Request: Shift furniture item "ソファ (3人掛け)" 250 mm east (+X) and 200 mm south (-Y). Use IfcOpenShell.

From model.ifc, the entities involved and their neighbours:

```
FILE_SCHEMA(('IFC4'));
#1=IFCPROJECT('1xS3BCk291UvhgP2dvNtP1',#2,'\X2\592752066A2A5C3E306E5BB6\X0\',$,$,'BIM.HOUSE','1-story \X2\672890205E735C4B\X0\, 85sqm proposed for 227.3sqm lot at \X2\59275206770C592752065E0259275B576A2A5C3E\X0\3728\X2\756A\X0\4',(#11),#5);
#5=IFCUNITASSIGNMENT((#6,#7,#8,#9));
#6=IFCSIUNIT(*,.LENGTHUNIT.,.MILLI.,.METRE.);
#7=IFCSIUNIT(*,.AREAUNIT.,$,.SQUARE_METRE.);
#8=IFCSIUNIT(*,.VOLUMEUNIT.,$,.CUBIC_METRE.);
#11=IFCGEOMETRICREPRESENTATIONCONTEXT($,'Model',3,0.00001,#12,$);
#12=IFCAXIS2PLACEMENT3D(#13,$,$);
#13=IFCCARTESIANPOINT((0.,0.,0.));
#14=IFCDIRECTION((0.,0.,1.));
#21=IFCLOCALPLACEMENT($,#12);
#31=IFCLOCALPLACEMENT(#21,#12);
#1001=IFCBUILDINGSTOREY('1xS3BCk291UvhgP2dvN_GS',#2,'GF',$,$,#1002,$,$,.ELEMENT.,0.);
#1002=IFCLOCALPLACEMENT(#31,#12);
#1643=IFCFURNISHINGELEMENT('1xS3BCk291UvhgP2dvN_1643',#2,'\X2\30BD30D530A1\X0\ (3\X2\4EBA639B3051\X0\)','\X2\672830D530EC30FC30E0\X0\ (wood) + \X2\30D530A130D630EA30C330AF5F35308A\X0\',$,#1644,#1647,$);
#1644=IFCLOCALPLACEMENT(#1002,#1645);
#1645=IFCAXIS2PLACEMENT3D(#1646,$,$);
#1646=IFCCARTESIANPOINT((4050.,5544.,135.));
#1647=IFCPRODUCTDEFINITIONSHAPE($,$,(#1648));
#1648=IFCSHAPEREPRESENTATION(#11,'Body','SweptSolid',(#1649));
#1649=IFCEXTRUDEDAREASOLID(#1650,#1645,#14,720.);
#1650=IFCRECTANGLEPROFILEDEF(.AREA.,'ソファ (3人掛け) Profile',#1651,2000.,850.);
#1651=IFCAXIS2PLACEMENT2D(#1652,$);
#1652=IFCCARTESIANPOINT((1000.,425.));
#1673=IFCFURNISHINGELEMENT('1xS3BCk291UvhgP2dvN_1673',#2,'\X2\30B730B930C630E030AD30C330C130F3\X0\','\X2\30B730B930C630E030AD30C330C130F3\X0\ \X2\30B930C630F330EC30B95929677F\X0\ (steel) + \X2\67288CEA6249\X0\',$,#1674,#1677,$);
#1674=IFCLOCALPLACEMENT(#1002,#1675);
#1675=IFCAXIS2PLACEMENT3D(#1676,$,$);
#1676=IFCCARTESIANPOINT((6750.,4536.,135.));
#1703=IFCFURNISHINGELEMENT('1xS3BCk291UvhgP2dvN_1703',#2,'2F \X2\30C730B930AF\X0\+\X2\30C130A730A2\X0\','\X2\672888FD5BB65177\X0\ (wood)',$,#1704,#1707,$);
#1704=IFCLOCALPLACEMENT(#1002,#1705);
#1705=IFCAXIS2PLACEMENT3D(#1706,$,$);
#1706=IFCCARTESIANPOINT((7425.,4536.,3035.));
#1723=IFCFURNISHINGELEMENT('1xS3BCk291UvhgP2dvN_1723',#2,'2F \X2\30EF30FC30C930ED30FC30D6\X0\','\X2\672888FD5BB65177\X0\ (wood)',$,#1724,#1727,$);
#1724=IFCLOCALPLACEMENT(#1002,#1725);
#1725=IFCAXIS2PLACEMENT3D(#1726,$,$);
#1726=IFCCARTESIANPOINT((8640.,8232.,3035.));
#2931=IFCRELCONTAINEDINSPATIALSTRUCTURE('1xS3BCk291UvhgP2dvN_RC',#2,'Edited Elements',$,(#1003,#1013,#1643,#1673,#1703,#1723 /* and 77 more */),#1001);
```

```python
import ifcopenshell
import ifcopenshell.api.geometry
import ifcopenshell.util.placement
import ifcopenshell.util.unit

model = ifcopenshell.open("model.ifc")
unit_scale = ifcopenshell.util.unit.calculate_unit_scale(model)

item = model.by_id(1643)
matrix = ifcopenshell.util.placement.get_local_placement(item.ObjectPlacement)
matrix[0, 3] += 0.25 / unit_scale
matrix[1, 3] -= 0.2 / unit_scale
ifcopenshell.api.geometry.edit_object_placement(model, product=item, matrix=matrix, is_si=False)

print(ifcopenshell.util.placement.get_local_placement(item.ObjectPlacement).round(3) + 0.0)

model.write("model_edited.ifc")
```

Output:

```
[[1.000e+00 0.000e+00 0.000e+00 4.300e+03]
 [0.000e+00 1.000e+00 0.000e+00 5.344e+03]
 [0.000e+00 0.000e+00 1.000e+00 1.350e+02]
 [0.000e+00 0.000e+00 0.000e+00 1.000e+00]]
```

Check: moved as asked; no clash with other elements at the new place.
